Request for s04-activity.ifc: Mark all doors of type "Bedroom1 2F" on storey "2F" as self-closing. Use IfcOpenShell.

First a look at what the model holds.

```python
import ifcopenshell
import ifcopenshell.util.element

model = ifcopenshell.open("s04-activity.ifc")
print(model.schema)
storey = next(s for s in model.by_type("IfcBuildingStorey") if s.Name == "2F")
doors = [e for e in ifcopenshell.util.element.get_decomposition(storey) if e.is_a("IfcDoor")]
seen = {}
for e in doors:
    element_type = ifcopenshell.util.element.get_type(e)
    key = (element_type.Name if element_type != e and element_type else None, ifcopenshell.util.element.get_pset(e, "Pset_DoorCommon", "SelfClosing"))
    seen[key] = seen.get(key, 0) + 1
for (name, value), count in sorted(seen.items(), key=str):
    print(count, "x", name, "|", value)
```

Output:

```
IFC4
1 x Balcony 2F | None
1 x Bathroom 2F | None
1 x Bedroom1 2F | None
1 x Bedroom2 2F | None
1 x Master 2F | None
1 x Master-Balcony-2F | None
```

```python
import ifcopenshell
import ifcopenshell.api.pset
import ifcopenshell.util.element

model = ifcopenshell.open("s04-activity.ifc")

storey = next(s for s in model.by_type("IfcBuildingStorey") if s.Name == "2F")
doors = [e for e in ifcopenshell.util.element.get_decomposition(storey) if e.is_a("IfcDoor")]

count = 0
for e in doors:
    element_type = ifcopenshell.util.element.get_type(e)
    if element_type in (None, e) or element_type.Name != "Bedroom1 2F":
        continue
    # add_pset returns the element's existing set when there is one.
    pset = ifcopenshell.api.pset.add_pset(model, product=e, name="Pset_DoorCommon")
    ifcopenshell.api.pset.edit_pset(model, pset=pset, properties={"SelfClosing": True})
    count += 1

print(count, "doors updated")

model.write("s04-activity_v2.ifc")
```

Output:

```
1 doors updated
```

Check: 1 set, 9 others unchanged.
